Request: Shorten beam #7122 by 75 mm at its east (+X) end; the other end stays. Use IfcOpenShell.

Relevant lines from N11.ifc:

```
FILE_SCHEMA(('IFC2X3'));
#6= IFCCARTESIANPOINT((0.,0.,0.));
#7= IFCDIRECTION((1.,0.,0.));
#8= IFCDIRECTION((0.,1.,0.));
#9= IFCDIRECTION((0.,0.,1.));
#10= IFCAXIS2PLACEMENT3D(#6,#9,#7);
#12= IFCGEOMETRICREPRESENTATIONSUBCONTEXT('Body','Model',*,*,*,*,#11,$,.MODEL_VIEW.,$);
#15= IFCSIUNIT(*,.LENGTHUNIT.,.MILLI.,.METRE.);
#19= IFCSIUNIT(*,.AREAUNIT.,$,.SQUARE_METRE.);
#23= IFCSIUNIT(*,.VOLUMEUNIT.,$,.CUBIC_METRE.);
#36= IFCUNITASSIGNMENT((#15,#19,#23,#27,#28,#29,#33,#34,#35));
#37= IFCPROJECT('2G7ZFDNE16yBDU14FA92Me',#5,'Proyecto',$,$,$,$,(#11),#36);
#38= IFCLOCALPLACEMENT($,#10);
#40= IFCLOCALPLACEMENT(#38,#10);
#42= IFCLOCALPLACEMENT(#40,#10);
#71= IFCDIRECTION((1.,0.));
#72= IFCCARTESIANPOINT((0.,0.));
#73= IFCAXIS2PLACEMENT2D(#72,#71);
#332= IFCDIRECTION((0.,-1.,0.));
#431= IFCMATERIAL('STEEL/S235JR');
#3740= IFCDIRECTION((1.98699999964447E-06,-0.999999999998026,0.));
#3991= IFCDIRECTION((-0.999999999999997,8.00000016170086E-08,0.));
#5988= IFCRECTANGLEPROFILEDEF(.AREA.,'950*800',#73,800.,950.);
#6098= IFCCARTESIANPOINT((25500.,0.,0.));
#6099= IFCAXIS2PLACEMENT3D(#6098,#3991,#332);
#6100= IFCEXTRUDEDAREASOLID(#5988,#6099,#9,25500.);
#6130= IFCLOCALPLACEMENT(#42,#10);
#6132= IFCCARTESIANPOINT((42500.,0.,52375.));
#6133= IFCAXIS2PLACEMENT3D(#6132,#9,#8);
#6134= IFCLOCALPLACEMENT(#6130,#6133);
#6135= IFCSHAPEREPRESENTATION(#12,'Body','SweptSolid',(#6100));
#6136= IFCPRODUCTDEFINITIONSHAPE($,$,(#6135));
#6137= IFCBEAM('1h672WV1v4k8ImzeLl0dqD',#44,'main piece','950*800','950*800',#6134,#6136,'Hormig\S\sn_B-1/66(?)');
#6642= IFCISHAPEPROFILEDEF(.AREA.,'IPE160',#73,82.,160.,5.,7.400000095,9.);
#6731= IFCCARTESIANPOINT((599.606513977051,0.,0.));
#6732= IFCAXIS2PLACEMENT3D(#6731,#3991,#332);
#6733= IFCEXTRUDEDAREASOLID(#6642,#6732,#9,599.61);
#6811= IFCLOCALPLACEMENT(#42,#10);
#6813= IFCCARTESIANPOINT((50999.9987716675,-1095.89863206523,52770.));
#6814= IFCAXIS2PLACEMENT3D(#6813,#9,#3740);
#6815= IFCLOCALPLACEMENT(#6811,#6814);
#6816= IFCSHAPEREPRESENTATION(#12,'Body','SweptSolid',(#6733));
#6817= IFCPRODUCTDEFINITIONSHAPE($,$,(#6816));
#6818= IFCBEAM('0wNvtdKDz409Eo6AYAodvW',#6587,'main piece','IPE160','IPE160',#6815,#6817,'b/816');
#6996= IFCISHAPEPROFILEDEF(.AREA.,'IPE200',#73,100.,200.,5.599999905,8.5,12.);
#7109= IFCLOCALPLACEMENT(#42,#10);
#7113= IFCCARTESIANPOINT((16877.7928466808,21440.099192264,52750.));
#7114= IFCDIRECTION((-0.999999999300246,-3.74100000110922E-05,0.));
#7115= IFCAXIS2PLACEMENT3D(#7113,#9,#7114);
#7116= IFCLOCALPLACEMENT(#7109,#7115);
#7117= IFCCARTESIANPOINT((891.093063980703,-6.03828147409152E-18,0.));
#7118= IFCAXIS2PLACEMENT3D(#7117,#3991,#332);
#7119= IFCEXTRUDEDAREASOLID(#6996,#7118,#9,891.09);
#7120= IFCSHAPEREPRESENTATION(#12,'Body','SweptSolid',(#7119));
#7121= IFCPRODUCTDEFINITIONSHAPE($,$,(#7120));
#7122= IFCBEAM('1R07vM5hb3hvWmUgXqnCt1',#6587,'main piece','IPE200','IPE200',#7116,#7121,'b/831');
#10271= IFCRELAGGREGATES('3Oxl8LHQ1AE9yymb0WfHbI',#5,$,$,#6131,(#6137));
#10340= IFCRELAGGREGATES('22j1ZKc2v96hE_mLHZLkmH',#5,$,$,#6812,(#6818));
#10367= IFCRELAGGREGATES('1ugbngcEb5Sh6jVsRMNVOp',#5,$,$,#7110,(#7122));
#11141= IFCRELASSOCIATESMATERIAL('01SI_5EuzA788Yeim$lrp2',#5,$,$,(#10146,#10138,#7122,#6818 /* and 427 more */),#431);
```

```python
import ifcopenshell
import ifcopenshell.util.representation
import ifcopenshell.util.unit

model = ifcopenshell.open("N11.ifc")
unit_scale = ifcopenshell.util.unit.calculate_unit_scale(model)

member = model.by_id(7122)
change = -0.075 / unit_scale

# The extrusion runs towards the end named, so only its depth changes.
body = ifcopenshell.util.representation.get_representation(member, "Model", "Body")
solid = body.Items[0]
old_length = solid.Depth
solid.Depth += change

print(f"length {old_length:g} -> {solid.Depth:g}")

model.write("N11_rev.ifc")
```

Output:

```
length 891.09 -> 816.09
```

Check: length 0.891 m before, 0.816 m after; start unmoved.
